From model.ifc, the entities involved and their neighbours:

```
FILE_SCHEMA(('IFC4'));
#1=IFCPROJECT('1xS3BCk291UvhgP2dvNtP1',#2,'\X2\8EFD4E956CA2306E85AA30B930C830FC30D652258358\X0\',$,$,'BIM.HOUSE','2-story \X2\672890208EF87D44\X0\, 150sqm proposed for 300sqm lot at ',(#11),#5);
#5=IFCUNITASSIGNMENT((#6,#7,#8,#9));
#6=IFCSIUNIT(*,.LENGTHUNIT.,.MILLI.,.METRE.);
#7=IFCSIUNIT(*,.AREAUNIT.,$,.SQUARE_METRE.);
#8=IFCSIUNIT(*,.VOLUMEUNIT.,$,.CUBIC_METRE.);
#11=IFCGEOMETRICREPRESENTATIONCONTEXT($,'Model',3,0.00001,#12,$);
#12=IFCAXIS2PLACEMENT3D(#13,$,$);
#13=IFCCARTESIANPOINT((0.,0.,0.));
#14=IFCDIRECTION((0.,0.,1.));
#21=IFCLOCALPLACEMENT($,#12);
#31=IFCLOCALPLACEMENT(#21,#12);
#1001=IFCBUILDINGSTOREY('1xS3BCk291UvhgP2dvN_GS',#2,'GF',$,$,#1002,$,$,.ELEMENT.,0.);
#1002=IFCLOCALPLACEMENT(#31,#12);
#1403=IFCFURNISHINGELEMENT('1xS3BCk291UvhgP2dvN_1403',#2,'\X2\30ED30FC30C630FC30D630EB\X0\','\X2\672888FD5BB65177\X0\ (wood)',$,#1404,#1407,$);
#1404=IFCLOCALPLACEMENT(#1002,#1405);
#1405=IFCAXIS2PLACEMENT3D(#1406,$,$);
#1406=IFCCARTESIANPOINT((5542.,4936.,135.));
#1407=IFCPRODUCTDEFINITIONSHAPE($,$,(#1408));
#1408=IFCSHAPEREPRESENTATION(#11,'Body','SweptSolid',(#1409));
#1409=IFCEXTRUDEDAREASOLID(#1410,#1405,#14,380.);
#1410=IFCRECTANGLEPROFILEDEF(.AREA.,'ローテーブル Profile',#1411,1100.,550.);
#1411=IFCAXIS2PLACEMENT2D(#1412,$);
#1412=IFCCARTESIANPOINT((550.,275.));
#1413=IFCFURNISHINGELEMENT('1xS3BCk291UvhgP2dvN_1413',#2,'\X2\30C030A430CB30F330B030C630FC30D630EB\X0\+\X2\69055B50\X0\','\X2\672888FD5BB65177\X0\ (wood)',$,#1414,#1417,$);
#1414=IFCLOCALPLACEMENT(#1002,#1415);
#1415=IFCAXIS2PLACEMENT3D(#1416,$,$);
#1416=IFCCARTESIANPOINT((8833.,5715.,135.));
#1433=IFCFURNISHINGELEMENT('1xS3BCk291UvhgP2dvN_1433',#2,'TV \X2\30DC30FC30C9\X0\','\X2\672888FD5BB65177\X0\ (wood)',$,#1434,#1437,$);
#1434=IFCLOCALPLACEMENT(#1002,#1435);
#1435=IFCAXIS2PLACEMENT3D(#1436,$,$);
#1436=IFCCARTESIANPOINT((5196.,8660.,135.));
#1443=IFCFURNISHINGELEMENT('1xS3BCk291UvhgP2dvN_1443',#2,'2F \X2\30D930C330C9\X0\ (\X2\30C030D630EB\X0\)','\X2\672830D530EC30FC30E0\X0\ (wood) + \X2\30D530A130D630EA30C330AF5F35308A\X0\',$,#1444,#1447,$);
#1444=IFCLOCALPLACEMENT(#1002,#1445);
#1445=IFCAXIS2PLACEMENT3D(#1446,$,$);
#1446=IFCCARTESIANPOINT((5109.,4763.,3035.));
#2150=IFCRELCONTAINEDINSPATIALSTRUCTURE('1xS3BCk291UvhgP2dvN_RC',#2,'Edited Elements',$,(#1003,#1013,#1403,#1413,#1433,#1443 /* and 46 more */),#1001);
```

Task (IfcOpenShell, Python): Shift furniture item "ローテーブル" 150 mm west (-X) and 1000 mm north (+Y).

```python
import ifcopenshell
import ifcopenshell.api.geometry
import ifcopenshell.util.placement
import ifcopenshell.util.unit

model = ifcopenshell.open("model.ifc")
unit_scale = ifcopenshell.util.unit.calculate_unit_scale(model)

item = model.by_guid("1xS3BCk291UvhgP2dvN_1403")
matrix = ifcopenshell.util.placement.get_local_placement(item.ObjectPlacement)
matrix[0, 3] -= 0.15 / unit_scale
matrix[1, 3] += 1 / unit_scale
ifcopenshell.api.geometry.edit_object_placement(model, product=item, matrix=matrix, is_si=False)

print(ifcopenshell.util.placement.get_local_placement(item.ObjectPlacement).round(3) + 0.0)

model.write("model-out.ifc")
```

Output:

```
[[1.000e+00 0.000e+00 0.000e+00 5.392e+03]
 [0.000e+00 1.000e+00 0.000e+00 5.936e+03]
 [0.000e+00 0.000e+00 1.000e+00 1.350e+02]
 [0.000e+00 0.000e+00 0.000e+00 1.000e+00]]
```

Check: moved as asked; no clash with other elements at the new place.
